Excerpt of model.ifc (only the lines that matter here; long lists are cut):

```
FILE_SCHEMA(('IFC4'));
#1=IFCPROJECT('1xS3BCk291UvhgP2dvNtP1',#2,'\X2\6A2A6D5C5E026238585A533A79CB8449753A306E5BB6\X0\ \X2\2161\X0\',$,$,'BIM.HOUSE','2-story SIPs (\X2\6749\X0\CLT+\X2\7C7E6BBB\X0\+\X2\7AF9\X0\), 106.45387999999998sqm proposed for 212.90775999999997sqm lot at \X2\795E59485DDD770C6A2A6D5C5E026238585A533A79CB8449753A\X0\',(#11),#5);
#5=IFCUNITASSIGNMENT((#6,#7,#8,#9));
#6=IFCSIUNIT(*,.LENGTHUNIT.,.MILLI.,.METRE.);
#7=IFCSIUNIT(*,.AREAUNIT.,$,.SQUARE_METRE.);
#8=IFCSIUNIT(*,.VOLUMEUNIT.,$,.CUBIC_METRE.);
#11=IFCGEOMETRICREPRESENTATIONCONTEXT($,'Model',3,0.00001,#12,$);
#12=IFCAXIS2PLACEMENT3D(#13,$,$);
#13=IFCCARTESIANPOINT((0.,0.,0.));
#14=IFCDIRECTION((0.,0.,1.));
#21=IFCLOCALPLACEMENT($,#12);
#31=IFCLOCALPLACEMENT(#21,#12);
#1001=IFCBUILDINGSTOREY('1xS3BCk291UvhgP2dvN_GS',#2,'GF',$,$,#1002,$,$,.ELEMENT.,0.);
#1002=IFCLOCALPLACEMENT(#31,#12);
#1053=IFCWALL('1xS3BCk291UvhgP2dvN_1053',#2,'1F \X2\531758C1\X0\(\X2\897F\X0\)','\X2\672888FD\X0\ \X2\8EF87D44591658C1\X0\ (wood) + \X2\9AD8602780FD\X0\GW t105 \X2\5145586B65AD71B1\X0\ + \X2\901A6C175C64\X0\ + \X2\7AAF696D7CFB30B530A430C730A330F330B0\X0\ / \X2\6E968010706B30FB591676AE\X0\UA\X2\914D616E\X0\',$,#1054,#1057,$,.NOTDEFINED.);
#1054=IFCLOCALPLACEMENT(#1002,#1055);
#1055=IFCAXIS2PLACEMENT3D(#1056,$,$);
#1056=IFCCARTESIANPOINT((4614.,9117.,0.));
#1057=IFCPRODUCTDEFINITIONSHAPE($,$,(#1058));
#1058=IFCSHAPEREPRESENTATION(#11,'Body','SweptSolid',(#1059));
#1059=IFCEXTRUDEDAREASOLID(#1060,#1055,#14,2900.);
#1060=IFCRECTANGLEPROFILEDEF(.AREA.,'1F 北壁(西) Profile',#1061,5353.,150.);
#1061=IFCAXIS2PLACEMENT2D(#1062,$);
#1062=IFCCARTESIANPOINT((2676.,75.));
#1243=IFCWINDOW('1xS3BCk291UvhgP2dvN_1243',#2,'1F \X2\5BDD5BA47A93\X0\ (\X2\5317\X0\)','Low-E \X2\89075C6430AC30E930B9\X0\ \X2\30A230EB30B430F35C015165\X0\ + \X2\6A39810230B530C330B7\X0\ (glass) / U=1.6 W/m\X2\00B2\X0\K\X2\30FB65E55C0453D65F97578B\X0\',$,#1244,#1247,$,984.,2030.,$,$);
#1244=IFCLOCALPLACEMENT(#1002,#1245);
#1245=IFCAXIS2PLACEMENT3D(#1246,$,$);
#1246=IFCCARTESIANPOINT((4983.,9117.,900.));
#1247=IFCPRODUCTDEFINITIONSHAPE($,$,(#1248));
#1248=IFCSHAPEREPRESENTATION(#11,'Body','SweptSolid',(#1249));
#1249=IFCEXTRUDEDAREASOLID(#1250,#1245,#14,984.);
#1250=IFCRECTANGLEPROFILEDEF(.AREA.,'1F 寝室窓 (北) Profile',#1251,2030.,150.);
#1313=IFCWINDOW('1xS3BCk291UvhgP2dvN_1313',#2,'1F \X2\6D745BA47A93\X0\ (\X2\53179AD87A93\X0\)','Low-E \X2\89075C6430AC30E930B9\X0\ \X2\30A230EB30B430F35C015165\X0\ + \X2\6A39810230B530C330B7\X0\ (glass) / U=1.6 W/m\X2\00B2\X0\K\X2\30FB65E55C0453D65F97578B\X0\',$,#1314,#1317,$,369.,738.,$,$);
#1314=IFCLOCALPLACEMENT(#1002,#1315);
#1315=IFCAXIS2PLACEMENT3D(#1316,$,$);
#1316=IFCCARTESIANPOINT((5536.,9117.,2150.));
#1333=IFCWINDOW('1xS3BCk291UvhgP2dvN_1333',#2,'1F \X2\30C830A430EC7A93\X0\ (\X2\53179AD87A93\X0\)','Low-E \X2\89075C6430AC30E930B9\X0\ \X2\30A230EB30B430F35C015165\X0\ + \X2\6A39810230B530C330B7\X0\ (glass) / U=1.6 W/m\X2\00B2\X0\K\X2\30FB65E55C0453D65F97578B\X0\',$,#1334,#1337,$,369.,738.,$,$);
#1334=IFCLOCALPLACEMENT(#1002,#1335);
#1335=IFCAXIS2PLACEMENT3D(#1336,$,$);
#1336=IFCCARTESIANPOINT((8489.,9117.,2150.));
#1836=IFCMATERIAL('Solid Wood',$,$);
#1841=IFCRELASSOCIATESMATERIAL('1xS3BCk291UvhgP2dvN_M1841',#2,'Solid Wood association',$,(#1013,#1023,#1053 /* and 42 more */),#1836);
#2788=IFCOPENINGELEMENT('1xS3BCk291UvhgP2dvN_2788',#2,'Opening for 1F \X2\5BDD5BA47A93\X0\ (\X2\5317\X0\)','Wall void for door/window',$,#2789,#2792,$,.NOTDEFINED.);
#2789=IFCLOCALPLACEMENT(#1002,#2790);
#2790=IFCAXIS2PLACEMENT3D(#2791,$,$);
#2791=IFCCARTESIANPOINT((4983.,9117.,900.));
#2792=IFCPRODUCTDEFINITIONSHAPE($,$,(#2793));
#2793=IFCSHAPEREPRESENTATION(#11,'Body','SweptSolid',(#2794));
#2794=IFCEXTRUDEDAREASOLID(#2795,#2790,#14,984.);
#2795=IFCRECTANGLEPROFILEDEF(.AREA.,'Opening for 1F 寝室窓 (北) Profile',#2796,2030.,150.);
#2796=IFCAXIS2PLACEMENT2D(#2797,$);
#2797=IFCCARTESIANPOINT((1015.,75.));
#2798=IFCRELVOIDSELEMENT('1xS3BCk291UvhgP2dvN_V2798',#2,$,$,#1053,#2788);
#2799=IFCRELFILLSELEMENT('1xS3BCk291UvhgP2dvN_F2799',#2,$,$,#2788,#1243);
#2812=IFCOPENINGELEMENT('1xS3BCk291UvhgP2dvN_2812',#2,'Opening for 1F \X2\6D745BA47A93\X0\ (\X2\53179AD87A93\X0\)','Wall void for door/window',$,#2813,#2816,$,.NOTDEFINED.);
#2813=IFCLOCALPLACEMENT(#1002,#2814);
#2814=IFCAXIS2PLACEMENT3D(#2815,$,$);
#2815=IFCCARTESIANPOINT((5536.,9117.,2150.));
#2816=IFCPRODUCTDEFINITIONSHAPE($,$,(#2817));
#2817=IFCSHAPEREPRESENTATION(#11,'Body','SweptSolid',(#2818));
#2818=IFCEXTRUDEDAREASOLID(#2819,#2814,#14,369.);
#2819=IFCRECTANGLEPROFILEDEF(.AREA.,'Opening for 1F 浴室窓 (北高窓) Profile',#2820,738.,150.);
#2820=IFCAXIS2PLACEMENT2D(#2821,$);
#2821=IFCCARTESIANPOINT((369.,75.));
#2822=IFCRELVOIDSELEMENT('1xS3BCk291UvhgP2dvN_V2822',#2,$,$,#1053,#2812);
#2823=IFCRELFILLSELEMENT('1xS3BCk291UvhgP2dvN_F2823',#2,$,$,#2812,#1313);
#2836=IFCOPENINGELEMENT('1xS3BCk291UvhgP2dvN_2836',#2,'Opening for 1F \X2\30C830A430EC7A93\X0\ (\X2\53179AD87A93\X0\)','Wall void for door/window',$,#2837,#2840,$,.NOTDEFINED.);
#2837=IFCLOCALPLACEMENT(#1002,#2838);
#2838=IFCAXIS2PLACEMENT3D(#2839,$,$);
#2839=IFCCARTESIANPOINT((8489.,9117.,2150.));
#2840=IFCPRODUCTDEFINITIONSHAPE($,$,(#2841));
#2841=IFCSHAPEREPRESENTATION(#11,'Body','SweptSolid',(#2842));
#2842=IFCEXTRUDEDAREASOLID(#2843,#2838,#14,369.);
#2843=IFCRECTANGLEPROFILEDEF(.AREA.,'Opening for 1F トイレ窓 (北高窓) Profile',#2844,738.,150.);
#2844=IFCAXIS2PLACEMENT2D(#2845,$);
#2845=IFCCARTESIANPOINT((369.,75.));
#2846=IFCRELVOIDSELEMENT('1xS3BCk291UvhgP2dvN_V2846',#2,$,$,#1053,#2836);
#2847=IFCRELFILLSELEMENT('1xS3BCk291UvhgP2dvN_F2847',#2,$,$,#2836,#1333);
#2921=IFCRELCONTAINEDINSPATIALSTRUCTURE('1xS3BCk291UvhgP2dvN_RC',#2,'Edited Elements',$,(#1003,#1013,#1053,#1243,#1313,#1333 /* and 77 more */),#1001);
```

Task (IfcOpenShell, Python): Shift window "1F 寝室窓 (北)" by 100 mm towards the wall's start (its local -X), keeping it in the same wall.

```python
import ifcopenshell
import ifcopenshell.api.geometry
import ifcopenshell.util.placement

model = ifcopenshell.open("model.ifc")

window = model.by_id(1243)
opening = window.FillsVoids[0].RelatingOpeningElement
wall = opening.VoidsElements[0].RelatingBuildingElement

wall_matrix = ifcopenshell.util.placement.get_local_placement(wall.ObjectPlacement)
shift = wall_matrix[:3, 0] * -100.0
before = ifcopenshell.util.placement.get_local_placement(window.ObjectPlacement)[:3, 3].copy()

# The window is not placed relative to its opening, so move both.
for product in (opening, window):
    matrix = ifcopenshell.util.placement.get_local_placement(product.ObjectPlacement)
    matrix[:3, 3] += shift
    ifcopenshell.api.geometry.edit_object_placement(model, product=product, matrix=matrix, is_si=False)

after = ifcopenshell.util.placement.get_local_placement(window.ObjectPlacement)[:3, 3]
print("window moved by", (after - before).round(3) + 0.0)

model.write("model_edited.ifc")
```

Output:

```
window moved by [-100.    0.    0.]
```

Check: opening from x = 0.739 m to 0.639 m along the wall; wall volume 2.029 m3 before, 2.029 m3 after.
